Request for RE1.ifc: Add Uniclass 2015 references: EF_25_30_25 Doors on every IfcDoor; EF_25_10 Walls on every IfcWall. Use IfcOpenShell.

First a look at what the model holds.

```python
import ifcopenshell

model = ifcopenshell.open("RE1.ifc")
print(model.schema)
print("classifications:", [c.Name for c in model.by_type("IfcClassification")])
for ifc_class in ("IfcDoor", "IfcRoof", "IfcStair", "IfcWall", "IfcWindow"):
    print(ifc_class, len(model.by_type(ifc_class)))
```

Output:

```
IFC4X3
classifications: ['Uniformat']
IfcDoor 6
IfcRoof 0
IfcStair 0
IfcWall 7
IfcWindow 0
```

```python
import ifcopenshell
import ifcopenshell.api.classification

model = ifcopenshell.open("RE1.ifc")

system = ifcopenshell.api.classification.add_classification(model, classification="Uniclass 2015")

codes = {
    "IfcDoor": ("EF_25_30_25", "Doors"),
    "IfcWall": ("EF_25_10", "Walls"),
}
for ifc_class, (code, name) in codes.items():
    products = model.by_type(ifc_class)
    ifcopenshell.api.classification.add_reference(
        model, products=products, classification=system, identification=code, name=name
    )
    print(code, len(products))

model.write("RE1_edited.ifc")
```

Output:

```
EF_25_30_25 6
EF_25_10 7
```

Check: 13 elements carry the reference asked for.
